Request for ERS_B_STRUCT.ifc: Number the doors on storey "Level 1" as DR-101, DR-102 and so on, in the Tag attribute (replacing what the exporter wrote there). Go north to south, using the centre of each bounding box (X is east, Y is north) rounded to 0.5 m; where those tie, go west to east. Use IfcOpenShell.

First a look at what the model holds.

```python
import ifcopenshell
import ifcopenshell.util.element
import ifcopenshell.util.placement

model = ifcopenshell.open("ERS_B_STRUCT.ifc")
print(model.schema)
storey = next(s for s in model.by_type("IfcBuildingStorey") if s.Name == "Level 1")
doors = [e for e in ifcopenshell.util.element.get_decomposition(storey) if e.is_a("IfcDoor")]
for e in sorted(doors, key=lambda e: e.id()):
    origin = ifcopenshell.util.placement.get_local_placement(e.ObjectPlacement)[:3, 3]
    print(e.id(), e.Tag, e.Name, origin.round(2) + 0.0, sep=" | ")
```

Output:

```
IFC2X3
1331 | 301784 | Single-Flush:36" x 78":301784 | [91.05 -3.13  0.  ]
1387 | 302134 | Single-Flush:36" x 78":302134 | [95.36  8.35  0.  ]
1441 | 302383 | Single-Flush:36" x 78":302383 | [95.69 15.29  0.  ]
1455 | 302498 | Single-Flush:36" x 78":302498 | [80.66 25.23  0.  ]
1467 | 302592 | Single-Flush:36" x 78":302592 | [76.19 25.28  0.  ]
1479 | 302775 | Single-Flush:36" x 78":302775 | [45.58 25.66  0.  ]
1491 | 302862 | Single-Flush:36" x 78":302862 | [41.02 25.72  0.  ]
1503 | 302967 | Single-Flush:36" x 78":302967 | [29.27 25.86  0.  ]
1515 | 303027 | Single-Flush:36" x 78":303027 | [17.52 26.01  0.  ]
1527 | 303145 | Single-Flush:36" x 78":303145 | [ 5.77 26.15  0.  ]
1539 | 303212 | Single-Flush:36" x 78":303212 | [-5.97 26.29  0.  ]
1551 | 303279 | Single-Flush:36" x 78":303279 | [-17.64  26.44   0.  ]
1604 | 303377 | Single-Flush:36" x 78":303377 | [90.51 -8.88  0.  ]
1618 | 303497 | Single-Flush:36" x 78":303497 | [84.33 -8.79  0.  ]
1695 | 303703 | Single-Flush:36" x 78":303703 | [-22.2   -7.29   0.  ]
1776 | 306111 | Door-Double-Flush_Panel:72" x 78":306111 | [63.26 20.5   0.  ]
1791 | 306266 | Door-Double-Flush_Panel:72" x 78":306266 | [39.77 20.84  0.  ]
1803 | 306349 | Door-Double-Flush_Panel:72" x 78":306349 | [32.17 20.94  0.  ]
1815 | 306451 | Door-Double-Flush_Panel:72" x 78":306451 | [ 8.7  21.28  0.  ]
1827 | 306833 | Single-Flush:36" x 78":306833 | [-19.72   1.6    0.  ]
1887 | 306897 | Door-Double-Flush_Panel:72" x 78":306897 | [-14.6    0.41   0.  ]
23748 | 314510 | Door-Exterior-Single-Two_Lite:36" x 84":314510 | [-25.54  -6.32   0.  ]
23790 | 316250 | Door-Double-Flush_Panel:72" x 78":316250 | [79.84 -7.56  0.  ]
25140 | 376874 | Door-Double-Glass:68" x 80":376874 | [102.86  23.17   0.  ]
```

```python
import ifcopenshell
import ifcopenshell.geom
import ifcopenshell.util.element
import ifcopenshell.util.shape

model = ifcopenshell.open("ERS_B_STRUCT.ifc")
settings = ifcopenshell.geom.settings()
settings.set("use-world-coords", True)


def centre(element):
    shape = ifcopenshell.geom.create_shape(settings, element)
    return ifcopenshell.util.shape.get_bbox_centroid(shape.geometry)


storey = next(s for s in model.by_type("IfcBuildingStorey") if s.Name == "Level 1")
doors = [e for e in ifcopenshell.util.element.get_decomposition(storey) if e.is_a("IfcDoor")]

# Insertion points can sit at a corner or the storey origin, so sort by the geometry (in metres).
centres = {e: centre(e) for e in doors}
doors.sort(key=lambda e: (-round(centres[e][1] / 0.5), centres[e][0]))

for i, e in enumerate(doors, start=1):
    number = f"DR-1{i:02d}"
    e.Tag = number
    print(e.id(), number)

model.write("ERS_B_STRUCT_v2.ifc")
```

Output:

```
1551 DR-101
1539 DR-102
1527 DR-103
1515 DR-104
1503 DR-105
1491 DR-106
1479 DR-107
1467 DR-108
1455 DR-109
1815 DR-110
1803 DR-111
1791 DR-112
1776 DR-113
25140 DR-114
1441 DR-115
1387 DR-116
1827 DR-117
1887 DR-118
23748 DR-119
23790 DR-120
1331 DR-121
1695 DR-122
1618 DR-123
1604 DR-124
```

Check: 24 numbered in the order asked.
